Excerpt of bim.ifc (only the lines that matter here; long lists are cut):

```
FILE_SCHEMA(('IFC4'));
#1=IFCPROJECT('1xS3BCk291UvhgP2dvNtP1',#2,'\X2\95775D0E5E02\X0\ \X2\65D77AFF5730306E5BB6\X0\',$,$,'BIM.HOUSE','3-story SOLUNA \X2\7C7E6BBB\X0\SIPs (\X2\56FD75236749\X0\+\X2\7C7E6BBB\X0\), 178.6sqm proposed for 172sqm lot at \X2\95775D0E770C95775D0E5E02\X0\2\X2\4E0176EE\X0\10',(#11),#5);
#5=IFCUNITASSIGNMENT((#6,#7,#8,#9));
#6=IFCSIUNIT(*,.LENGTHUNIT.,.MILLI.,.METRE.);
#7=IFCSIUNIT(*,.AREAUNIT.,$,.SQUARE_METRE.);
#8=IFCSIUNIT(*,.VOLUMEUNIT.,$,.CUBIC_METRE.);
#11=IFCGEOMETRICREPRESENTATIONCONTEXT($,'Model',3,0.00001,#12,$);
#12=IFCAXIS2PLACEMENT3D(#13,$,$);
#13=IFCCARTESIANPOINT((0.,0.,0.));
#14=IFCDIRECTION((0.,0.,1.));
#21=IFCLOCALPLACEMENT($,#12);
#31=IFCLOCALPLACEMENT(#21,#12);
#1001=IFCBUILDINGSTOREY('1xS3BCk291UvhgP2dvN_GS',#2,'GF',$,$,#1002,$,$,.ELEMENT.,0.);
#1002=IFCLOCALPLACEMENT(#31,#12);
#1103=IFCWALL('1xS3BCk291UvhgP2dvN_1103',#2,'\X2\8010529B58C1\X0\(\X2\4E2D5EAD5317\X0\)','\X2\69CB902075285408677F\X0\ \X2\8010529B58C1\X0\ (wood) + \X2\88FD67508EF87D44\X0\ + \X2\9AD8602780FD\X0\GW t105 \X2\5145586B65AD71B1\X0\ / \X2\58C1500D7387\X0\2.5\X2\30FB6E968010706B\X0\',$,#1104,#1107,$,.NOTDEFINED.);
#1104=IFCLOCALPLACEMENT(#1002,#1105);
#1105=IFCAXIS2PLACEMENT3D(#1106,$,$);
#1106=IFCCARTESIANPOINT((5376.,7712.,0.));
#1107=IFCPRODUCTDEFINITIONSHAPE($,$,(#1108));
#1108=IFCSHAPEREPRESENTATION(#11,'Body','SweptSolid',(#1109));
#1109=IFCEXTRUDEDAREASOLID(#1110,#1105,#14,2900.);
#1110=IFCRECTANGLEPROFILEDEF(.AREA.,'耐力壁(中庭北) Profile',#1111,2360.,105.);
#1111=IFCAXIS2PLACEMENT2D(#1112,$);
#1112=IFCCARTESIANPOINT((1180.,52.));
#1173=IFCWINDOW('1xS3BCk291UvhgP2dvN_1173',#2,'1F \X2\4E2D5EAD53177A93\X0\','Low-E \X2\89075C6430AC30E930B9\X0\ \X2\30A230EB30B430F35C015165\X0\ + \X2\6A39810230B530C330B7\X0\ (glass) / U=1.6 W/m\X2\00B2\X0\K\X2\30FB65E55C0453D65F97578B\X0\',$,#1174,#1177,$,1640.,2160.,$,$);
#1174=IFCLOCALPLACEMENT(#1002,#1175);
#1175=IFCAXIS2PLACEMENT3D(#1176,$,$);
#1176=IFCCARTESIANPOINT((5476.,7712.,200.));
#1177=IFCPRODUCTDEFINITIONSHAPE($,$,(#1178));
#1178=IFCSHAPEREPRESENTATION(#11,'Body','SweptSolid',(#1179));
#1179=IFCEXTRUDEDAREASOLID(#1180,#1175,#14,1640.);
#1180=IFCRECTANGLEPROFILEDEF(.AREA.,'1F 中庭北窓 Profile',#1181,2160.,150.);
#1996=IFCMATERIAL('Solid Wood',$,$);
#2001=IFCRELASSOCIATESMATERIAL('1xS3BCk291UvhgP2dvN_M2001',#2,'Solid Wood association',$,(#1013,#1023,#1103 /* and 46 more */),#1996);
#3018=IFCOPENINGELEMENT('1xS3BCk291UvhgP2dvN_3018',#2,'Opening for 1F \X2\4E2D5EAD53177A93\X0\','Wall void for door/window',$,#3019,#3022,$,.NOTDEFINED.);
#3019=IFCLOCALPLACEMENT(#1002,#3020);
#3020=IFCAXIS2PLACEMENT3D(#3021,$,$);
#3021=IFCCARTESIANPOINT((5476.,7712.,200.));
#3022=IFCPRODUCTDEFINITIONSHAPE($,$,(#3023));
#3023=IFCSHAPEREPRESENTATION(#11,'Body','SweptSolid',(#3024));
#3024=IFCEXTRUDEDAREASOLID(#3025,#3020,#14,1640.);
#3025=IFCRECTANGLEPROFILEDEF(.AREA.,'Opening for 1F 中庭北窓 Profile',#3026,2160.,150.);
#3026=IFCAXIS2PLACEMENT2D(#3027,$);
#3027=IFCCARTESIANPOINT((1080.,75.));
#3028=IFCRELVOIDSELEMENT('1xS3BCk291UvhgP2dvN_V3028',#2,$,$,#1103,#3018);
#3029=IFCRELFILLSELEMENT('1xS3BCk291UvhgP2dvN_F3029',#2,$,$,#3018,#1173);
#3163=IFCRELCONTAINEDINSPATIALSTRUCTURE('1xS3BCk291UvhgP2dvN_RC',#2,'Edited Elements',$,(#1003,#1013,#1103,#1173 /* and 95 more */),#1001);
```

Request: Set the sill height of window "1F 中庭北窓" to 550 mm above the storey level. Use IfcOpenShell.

```python
import numpy as np
import ifcopenshell
import ifcopenshell.api.geometry
import ifcopenshell.geom
import ifcopenshell.util.element
import ifcopenshell.util.placement
import ifcopenshell.util.shape
import ifcopenshell.util.unit

model = ifcopenshell.open("bim.ifc")
unit_scale = ifcopenshell.util.unit.calculate_unit_scale(model)

window = model.by_guid("1xS3BCk291UvhgP2dvN_1173")
opening = window.FillsVoids[0].RelatingOpeningElement
storey = ifcopenshell.util.element.get_container(window, ifc_class="IfcBuildingStorey")
level = ifcopenshell.util.placement.get_local_placement(storey.ObjectPlacement)[2, 3]

# The opening's origin need not be at the sill, so measure its lowest point.
shape = ifcopenshell.geom.create_shape(ifcopenshell.geom.settings(), opening)
bottom = ifcopenshell.util.shape.get_shape_bottom_elevation(shape, shape.geometry) / unit_scale
dz = level + 550.0 - bottom

shift = np.array([0.0, 0.0, dz])
# The window is not placed relative to its opening, so move both.
for product in (opening, window):
    matrix = ifcopenshell.util.placement.get_local_placement(product.ObjectPlacement)
    matrix[:3, 3] += shift
    ifcopenshell.api.geometry.edit_object_placement(model, product=product, matrix=matrix, is_si=False)

print(f"moved by {dz * unit_scale:+.3f} m")

model.write("bim_v2.ifc")
```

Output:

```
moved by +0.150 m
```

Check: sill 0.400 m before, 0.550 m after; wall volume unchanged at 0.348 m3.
